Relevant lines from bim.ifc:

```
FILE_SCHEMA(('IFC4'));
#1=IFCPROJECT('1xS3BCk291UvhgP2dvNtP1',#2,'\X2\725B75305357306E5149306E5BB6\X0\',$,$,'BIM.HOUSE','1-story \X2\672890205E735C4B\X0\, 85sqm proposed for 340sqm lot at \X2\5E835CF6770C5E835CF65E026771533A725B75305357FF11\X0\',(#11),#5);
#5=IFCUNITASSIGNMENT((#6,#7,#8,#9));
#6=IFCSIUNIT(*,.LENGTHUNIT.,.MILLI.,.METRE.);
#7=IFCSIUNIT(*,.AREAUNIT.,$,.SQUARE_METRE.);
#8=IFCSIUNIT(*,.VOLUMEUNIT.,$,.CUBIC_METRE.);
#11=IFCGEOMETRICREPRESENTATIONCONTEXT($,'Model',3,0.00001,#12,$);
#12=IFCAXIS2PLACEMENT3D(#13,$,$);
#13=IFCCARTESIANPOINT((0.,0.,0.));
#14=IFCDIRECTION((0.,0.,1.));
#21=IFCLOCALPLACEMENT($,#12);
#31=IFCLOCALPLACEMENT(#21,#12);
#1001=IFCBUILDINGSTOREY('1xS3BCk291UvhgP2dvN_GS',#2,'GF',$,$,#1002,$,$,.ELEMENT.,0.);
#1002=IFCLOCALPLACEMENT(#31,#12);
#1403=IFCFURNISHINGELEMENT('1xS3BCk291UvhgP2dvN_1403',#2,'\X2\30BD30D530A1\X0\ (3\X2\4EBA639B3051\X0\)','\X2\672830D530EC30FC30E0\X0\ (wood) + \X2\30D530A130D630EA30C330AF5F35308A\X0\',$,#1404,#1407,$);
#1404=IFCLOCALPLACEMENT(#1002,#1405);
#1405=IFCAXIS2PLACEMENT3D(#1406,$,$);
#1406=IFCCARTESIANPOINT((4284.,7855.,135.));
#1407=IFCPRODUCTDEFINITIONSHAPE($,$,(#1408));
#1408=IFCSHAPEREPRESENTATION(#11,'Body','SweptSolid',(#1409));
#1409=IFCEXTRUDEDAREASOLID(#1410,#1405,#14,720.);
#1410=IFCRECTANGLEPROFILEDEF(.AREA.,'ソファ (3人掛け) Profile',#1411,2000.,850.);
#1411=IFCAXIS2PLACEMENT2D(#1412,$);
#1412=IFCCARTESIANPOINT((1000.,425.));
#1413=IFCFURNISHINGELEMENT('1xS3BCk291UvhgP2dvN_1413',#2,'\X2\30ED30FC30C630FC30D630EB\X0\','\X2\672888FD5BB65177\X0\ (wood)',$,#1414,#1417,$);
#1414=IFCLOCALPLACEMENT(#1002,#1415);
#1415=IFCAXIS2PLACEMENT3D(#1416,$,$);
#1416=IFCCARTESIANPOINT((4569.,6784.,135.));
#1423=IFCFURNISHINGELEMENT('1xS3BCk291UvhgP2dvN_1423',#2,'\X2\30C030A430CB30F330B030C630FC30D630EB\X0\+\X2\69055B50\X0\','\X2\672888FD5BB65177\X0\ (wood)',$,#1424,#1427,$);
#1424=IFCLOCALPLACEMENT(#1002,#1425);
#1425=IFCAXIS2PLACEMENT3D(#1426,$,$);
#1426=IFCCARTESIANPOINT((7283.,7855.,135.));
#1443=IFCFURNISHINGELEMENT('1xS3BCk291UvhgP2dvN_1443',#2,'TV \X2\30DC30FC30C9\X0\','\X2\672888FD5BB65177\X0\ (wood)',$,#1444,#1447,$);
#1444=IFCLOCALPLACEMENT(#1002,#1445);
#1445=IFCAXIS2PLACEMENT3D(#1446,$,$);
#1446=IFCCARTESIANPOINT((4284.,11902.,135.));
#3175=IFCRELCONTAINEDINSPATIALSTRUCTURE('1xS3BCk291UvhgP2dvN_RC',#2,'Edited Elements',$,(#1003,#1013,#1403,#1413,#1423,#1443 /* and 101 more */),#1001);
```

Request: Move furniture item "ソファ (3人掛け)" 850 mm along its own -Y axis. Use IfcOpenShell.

```python
import ifcopenshell
import ifcopenshell.api.geometry
import ifcopenshell.util.placement
import ifcopenshell.util.unit

model = ifcopenshell.open("bim.ifc")
unit_scale = ifcopenshell.util.unit.calculate_unit_scale(model)

item = model.by_guid("1xS3BCk291UvhgP2dvN_1403")
matrix = ifcopenshell.util.placement.get_local_placement(item.ObjectPlacement)
matrix[:3, 3] -= matrix[:3, 1] * 0.85 / unit_scale
ifcopenshell.api.geometry.edit_object_placement(model, product=item, matrix=matrix, is_si=False)

print(ifcopenshell.util.placement.get_local_placement(item.ObjectPlacement).round(3) + 0.0)

model.write("bim_edited.ifc")
```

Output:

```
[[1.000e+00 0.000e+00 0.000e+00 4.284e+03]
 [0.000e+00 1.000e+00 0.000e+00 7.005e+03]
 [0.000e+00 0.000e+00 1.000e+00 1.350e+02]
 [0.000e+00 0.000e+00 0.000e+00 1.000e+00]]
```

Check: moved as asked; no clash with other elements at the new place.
